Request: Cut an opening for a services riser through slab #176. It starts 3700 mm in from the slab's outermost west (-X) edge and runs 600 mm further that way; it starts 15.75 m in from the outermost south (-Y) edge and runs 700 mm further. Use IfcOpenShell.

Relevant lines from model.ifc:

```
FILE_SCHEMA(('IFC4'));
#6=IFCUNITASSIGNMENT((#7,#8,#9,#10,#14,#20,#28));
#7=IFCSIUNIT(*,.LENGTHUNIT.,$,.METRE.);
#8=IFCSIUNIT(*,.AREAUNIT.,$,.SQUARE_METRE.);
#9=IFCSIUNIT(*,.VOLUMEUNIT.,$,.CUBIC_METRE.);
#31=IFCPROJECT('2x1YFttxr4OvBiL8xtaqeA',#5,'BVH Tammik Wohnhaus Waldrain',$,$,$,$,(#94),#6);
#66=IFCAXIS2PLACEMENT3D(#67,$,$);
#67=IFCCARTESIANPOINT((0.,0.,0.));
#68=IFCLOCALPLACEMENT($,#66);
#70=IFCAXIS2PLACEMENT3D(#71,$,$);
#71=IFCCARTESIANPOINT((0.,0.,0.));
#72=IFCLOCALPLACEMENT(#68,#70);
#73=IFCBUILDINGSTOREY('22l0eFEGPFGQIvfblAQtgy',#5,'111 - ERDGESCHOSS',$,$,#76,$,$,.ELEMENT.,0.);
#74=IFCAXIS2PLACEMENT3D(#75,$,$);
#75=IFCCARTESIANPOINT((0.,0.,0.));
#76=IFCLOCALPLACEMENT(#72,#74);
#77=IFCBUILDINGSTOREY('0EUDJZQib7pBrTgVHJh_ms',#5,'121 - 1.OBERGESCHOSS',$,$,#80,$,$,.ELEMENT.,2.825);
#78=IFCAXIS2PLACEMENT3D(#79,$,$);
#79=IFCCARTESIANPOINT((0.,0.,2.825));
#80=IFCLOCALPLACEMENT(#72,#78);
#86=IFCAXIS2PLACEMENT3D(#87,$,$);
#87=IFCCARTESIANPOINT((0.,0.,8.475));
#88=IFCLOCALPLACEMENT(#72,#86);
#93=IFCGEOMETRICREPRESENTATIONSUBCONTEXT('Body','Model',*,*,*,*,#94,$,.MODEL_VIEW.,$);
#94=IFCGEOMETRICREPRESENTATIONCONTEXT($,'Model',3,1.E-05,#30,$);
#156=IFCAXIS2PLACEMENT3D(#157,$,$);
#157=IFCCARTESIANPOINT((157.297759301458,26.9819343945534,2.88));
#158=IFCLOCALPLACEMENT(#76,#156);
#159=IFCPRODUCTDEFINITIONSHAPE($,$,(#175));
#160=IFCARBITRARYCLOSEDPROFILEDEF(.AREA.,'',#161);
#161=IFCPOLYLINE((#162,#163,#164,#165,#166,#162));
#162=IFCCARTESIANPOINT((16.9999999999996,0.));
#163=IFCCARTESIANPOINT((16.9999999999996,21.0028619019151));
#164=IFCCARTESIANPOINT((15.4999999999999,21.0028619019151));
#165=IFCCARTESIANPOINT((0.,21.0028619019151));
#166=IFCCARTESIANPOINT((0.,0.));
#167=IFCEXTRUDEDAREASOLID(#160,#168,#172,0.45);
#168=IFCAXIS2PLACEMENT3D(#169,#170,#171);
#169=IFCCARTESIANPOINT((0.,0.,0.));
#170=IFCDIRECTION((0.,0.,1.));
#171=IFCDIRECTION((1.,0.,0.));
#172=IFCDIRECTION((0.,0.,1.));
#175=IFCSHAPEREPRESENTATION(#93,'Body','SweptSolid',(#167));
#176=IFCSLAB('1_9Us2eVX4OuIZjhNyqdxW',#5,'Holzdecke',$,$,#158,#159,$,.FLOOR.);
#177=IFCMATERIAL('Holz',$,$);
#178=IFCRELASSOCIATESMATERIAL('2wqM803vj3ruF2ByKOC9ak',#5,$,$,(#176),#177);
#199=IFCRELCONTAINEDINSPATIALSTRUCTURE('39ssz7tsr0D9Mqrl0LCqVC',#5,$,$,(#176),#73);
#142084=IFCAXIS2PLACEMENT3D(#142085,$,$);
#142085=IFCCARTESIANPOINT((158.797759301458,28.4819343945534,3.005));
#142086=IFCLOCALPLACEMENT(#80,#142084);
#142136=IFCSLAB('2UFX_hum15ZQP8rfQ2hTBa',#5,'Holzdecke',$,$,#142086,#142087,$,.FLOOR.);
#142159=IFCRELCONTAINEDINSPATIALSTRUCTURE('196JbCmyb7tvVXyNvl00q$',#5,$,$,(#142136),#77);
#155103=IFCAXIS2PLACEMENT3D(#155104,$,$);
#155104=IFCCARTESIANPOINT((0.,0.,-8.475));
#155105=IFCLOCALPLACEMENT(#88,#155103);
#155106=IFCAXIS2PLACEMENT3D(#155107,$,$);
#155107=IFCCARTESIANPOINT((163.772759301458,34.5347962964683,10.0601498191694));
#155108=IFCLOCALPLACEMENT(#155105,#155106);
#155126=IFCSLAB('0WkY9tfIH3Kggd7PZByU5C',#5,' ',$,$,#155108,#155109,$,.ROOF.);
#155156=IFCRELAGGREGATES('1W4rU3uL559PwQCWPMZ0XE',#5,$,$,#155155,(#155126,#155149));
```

```python
import numpy as np
import ifcopenshell
import ifcopenshell.api.feature
import ifcopenshell.api.geometry
import ifcopenshell.api.root
import ifcopenshell.geom
import ifcopenshell.util.placement
import ifcopenshell.util.representation
import ifcopenshell.util.shape
import ifcopenshell.util.unit

model = ifcopenshell.open("model.ifc")
unit_scale = ifcopenshell.util.unit.calculate_unit_scale(model)
settings = ifcopenshell.geom.settings()


def volume(element):
    """Net volume in cubic metres, openings subtracted."""
    shape = ifcopenshell.geom.create_shape(settings, element)
    return ifcopenshell.util.shape.get_volume(shape.geometry)


slab = model.by_guid("1_9Us2eVX4OuIZjhNyqdxW")
before = volume(slab)

# Extent in the slab's own axes, in metres. The edges named are its -X and -Y sides.
slab_shape = ifcopenshell.geom.create_shape(settings, slab)
vertices = ifcopenshell.util.shape.get_vertices(slab_shape.geometry)
x_min, y_min, bottom = vertices.min(axis=0)
top = vertices[:, 2].max()

opening = ifcopenshell.api.root.create_entity(model, ifc_class="IfcOpeningElement", name="Services riser opening", predefined_type="OPENING")
context = ifcopenshell.util.representation.get_context(model, "Model", "Body", "MODEL_VIEW")
width, depth = 0.6, 0.7
outline = [(0.0, 0.0), (width, 0.0), (width, depth), (0.0, depth), (0.0, 0.0)]
# Overshoot both faces by 50 mm so the cut is clean.
shape = ifcopenshell.api.geometry.add_slab_representation(
    model, context=context, depth=top - bottom + 0.1, polyline=outline
)
ifcopenshell.api.geometry.assign_representation(model, product=opening, representation=shape)

matrix = ifcopenshell.util.placement.get_local_placement(slab.ObjectPlacement)
matrix[:, 3] = matrix @ np.append(np.array([x_min + 3.7, y_min + 15.75, bottom - 0.05]) / unit_scale, 1.0)
ifcopenshell.api.geometry.edit_object_placement(model, product=opening, matrix=matrix, is_si=False)
ifcopenshell.api.feature.add_feature(model, feature=opening, element=slab)

after = volume(slab)

print(f"slab volume {before:.3f} -> {after:.3f} m3")

model.write("model_edited.ifc")
```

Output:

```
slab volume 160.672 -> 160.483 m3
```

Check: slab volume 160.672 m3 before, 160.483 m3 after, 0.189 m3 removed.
